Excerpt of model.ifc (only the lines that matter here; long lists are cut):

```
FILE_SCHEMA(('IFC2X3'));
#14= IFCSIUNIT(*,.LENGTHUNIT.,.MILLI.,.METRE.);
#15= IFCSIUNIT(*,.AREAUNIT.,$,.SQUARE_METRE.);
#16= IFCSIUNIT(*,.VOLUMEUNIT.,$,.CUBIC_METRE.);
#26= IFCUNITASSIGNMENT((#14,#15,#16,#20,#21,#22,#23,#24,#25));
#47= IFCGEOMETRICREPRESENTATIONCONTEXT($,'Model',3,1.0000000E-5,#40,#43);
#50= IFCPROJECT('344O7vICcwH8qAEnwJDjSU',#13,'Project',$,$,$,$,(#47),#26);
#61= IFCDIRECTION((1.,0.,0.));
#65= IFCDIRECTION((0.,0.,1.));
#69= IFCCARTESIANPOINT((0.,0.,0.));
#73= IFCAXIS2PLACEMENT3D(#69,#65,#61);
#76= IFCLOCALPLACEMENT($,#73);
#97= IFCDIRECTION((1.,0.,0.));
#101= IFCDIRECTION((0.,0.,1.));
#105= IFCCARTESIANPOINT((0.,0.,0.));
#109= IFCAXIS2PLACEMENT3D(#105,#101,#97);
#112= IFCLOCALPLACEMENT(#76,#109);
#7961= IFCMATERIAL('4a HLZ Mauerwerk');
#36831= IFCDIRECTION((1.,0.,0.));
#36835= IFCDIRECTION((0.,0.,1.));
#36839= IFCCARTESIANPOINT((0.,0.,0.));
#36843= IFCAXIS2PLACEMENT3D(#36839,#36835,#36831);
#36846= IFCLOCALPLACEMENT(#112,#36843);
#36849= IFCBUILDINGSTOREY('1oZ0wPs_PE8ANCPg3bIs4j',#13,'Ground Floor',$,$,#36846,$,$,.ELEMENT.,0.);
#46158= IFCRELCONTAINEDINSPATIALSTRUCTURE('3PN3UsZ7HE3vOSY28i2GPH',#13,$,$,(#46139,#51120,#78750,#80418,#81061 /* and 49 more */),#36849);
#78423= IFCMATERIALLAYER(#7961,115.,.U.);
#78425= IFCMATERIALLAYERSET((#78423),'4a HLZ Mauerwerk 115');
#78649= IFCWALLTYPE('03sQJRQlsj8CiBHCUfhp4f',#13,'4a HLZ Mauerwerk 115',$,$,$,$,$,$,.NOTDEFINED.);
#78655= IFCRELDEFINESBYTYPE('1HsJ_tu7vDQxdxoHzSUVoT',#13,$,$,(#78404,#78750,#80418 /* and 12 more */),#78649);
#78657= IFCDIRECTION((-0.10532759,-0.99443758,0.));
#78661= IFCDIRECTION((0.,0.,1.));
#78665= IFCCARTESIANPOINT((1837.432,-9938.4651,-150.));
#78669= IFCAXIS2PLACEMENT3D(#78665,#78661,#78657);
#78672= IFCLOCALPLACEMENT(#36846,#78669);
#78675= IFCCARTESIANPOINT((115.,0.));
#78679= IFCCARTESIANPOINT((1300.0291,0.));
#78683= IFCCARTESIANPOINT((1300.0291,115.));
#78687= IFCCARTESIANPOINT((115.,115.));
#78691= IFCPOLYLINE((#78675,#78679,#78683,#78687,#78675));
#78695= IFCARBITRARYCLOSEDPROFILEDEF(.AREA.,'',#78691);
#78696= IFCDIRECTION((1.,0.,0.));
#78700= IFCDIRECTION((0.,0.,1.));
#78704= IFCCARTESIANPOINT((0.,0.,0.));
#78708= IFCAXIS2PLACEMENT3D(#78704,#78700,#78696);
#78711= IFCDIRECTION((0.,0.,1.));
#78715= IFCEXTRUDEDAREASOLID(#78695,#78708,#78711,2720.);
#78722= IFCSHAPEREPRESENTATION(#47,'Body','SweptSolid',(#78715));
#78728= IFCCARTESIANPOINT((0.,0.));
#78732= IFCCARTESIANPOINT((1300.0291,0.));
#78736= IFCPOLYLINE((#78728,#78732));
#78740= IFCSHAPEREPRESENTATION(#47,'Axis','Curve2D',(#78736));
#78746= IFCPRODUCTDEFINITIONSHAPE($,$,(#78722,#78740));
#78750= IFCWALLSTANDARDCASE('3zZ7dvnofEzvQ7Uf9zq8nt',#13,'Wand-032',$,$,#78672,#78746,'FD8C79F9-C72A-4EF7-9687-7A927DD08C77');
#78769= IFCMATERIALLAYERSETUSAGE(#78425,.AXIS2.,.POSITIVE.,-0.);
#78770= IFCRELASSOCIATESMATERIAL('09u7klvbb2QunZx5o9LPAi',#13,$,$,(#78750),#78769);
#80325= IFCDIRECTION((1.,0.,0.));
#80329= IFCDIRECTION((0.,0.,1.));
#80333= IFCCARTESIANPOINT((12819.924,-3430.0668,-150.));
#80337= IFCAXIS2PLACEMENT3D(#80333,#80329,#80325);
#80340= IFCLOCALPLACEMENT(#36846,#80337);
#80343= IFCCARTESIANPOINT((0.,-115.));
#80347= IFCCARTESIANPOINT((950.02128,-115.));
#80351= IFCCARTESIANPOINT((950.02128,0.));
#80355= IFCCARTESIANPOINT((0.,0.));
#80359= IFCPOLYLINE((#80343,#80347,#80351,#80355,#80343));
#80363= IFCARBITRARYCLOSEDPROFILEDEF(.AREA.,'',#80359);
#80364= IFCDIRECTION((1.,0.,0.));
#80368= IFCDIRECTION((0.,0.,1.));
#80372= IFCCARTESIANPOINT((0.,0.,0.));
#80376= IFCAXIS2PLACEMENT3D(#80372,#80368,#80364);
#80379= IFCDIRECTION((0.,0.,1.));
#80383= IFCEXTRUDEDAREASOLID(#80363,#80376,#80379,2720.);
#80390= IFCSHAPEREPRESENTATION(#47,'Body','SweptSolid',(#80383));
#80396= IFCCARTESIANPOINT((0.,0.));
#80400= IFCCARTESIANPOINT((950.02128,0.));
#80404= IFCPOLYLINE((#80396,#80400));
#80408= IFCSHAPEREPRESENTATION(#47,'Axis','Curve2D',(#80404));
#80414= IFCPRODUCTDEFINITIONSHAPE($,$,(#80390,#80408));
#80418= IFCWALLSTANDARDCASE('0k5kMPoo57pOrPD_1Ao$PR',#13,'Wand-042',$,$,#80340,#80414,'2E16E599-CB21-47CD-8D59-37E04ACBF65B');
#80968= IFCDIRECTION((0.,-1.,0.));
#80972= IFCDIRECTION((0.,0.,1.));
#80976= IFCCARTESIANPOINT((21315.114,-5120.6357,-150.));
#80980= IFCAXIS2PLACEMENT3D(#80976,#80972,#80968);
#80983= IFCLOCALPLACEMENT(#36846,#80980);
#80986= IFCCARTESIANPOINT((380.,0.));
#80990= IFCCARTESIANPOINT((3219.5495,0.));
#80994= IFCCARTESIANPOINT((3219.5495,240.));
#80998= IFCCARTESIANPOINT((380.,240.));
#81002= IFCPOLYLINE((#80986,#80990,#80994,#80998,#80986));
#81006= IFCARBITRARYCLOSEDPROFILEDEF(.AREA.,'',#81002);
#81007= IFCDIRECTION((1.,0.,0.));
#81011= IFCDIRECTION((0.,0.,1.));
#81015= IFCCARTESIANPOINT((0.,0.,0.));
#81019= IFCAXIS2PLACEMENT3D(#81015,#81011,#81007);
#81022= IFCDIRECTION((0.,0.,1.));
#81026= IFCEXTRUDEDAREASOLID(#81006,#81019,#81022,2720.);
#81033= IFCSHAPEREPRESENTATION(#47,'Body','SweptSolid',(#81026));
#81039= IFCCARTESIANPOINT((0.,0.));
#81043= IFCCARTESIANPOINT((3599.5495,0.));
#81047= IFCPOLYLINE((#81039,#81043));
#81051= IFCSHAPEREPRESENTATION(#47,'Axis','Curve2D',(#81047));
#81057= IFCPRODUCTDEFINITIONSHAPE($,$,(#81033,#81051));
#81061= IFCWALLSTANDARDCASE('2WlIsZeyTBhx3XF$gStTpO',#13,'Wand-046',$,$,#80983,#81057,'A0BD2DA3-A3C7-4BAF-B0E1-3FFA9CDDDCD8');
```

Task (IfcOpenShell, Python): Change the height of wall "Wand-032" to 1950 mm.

```python
import ifcopenshell
import ifcopenshell.geom
import ifcopenshell.util.shape
import ifcopenshell.util.unit

model = ifcopenshell.open("model.ifc")
unit_scale = ifcopenshell.util.unit.calculate_unit_scale(model)
settings = ifcopenshell.geom.settings()


def volume(element):
    """Net volume in cubic metres, openings subtracted."""
    shape = ifcopenshell.geom.create_shape(settings, element)
    return ifcopenshell.util.shape.get_volume(shape.geometry)


wall = model.by_id(78750)
before = volume(wall)

body = next(r for r in wall.Representation.Representations if r.RepresentationIdentifier == "Body")
solid = body.Items[0]
old_height = solid.Depth
solid.Depth = 1.95 / unit_scale
after = volume(wall)

print(f"height {old_height:g} -> {solid.Depth:g}, volume {before:.3f} -> {after:.3f} m3")

model.write("model_v2.ifc")
```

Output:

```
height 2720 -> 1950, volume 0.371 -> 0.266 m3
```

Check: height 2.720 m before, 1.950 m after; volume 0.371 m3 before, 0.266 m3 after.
